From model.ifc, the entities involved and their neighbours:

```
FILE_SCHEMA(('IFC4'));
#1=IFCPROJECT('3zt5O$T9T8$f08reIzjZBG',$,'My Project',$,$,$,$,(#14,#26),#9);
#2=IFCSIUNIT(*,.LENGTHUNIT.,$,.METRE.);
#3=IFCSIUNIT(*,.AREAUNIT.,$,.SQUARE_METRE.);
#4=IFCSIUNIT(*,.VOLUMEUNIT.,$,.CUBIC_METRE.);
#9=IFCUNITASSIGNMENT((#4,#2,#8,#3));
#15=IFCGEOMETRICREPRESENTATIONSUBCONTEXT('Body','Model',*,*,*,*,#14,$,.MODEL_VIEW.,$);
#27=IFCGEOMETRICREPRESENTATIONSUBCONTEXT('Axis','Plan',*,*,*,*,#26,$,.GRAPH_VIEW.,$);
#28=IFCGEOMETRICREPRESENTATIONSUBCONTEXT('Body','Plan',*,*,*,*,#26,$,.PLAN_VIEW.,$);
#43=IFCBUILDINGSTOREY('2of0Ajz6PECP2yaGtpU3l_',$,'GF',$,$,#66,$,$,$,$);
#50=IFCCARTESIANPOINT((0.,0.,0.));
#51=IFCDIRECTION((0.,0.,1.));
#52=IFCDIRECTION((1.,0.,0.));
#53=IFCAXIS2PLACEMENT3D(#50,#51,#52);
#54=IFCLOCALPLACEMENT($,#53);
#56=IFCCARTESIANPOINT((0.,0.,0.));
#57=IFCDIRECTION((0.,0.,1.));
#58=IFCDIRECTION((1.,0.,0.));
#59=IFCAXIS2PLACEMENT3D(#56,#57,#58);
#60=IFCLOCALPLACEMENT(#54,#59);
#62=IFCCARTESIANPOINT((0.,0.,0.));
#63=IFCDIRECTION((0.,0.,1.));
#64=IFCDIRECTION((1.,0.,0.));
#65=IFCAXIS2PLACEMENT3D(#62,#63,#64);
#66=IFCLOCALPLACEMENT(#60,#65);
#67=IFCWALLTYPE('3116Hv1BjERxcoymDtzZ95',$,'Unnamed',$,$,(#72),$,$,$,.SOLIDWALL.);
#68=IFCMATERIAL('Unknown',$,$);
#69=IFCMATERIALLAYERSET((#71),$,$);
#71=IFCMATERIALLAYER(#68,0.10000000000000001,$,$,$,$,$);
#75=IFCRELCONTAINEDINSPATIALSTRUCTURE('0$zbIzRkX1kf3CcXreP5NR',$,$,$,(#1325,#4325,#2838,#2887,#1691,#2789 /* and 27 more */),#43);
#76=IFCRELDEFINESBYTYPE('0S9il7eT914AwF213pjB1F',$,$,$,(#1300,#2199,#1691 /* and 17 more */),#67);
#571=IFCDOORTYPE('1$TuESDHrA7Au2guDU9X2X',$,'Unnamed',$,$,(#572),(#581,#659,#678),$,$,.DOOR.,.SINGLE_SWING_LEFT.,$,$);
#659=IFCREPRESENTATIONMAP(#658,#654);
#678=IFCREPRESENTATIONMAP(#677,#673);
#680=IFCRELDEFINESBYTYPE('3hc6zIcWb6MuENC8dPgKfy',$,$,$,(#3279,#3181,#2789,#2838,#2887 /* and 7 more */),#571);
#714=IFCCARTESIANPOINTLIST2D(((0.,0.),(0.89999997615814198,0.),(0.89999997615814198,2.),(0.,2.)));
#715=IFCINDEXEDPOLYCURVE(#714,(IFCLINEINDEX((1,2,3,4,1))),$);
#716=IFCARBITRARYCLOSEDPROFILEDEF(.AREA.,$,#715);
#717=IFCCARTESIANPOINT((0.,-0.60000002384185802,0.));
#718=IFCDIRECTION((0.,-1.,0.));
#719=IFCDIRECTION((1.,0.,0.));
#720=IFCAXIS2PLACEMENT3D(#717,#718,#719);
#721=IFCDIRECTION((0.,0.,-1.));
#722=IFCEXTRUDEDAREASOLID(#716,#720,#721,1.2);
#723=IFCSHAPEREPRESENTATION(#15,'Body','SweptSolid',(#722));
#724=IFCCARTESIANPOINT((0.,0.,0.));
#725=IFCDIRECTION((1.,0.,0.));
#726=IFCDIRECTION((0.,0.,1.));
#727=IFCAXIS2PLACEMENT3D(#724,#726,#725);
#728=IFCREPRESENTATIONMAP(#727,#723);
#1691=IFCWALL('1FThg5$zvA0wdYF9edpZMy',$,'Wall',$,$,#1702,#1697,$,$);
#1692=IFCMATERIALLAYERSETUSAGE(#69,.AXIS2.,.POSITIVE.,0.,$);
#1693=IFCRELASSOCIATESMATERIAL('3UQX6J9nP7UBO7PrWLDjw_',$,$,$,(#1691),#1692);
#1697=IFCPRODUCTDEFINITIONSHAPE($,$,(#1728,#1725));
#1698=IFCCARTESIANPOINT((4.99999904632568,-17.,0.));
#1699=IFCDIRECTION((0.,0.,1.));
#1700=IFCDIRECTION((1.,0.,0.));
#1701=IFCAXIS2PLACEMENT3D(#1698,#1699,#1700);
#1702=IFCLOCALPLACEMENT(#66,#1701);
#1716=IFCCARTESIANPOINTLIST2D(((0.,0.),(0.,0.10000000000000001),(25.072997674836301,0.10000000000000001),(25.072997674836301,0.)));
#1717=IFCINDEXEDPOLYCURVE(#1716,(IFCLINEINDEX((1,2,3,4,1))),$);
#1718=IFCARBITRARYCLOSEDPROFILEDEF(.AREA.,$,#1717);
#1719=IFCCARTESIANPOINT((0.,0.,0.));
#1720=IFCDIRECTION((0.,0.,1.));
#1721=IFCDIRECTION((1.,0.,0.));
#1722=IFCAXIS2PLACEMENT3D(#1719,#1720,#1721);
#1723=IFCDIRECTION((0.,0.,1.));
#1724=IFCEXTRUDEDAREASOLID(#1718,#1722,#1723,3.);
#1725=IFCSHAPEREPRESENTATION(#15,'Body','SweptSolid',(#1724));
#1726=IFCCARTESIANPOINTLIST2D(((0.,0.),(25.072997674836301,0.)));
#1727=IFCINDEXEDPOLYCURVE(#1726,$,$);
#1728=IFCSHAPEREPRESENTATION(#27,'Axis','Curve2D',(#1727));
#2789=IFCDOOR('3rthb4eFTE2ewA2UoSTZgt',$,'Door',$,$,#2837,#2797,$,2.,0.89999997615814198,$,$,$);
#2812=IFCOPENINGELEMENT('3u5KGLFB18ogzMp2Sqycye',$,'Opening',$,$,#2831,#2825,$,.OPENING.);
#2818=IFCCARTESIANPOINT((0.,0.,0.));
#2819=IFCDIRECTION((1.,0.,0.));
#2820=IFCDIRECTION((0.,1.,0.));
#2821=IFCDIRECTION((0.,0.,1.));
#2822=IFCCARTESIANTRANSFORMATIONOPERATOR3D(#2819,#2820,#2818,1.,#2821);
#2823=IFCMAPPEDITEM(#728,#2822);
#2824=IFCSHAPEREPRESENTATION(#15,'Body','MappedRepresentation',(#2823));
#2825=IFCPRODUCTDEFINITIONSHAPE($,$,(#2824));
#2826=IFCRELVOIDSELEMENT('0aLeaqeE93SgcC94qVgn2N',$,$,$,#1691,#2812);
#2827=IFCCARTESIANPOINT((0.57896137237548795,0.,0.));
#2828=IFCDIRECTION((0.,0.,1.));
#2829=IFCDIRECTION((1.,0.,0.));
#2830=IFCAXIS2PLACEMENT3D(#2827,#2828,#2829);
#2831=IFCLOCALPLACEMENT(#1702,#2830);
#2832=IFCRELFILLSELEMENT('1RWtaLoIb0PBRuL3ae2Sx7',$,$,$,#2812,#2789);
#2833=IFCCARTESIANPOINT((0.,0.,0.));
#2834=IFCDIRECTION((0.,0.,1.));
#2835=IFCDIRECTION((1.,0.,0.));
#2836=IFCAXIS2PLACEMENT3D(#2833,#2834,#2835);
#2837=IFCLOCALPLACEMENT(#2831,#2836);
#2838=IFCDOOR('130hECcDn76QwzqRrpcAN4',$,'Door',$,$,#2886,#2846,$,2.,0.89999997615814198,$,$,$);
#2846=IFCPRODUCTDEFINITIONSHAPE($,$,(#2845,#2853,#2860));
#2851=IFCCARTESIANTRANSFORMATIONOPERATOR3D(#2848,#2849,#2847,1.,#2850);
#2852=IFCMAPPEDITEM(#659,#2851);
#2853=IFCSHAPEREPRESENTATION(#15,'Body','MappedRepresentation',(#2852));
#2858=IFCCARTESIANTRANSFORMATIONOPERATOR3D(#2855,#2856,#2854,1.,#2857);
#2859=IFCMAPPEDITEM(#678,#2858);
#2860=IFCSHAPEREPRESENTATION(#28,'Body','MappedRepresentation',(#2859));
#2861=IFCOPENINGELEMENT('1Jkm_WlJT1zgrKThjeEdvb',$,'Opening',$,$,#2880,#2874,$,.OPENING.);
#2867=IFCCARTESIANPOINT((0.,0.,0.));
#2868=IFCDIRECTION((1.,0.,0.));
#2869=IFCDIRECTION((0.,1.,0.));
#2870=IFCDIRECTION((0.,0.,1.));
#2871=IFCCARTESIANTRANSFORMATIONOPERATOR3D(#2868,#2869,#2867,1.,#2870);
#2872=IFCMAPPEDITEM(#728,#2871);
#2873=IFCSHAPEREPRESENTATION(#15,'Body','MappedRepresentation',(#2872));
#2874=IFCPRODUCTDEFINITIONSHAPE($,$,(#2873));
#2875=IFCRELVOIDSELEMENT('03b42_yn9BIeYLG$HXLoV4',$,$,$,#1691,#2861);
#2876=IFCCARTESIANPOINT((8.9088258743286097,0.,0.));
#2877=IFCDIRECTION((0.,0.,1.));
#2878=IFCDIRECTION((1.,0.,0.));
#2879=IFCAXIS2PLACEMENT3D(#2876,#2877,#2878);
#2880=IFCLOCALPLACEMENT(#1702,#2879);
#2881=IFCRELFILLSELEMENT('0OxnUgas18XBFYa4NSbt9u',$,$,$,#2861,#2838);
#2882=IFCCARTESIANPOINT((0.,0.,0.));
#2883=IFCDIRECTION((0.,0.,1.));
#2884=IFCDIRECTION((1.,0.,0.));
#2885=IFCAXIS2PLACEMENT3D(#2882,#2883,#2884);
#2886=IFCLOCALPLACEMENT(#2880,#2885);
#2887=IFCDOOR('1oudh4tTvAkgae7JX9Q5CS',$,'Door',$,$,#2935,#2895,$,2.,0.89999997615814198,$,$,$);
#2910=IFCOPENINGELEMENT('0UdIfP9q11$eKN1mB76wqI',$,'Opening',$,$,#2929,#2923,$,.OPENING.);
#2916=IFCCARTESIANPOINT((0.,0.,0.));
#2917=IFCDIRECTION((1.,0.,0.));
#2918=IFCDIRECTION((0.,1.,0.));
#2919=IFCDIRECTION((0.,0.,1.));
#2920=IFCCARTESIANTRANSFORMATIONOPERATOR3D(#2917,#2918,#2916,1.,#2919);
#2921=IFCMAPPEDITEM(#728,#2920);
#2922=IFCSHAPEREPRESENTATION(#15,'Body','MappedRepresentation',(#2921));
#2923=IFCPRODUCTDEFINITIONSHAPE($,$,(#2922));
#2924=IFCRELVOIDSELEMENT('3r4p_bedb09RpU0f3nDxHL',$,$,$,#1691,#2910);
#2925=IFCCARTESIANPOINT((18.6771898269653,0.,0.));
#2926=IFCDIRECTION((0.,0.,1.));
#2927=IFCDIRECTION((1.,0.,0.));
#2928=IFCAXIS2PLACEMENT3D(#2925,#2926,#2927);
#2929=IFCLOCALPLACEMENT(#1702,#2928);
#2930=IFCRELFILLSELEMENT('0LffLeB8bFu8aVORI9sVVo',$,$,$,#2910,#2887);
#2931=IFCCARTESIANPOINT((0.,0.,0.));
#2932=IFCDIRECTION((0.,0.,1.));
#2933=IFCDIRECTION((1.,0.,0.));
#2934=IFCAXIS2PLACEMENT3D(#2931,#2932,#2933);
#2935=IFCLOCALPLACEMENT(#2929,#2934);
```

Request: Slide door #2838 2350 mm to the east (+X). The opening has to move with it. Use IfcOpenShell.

```python
import ifcopenshell
import ifcopenshell.api.geometry
import ifcopenshell.util.placement
import ifcopenshell.util.unit

model = ifcopenshell.open("model.ifc")
unit_scale = ifcopenshell.util.unit.calculate_unit_scale(model)

door = model.by_id(2838)
opening = door.FillsVoids[0].RelatingOpeningElement
wall = opening.VoidsElements[0].RelatingBuildingElement

wall_matrix = ifcopenshell.util.placement.get_local_placement(wall.ObjectPlacement)
shift = wall_matrix[:3, 0] * 2.35 / unit_scale
before = ifcopenshell.util.placement.get_local_placement(door.ObjectPlacement)[:3, 3].copy()

# The door is placed relative to its opening, so it follows when the opening moves.
matrix = ifcopenshell.util.placement.get_local_placement(opening.ObjectPlacement)
matrix[:3, 3] += shift
ifcopenshell.api.geometry.edit_object_placement(
    model, product=opening, matrix=matrix, is_si=False, should_transform_children=True
)

after = ifcopenshell.util.placement.get_local_placement(door.ObjectPlacement)[:3, 3]
print("door moved by", (after - before).round(3) + 0.0)

model.write("model_updated.ifc")
```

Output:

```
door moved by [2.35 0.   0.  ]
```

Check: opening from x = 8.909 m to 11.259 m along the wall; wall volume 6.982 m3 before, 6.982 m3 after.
